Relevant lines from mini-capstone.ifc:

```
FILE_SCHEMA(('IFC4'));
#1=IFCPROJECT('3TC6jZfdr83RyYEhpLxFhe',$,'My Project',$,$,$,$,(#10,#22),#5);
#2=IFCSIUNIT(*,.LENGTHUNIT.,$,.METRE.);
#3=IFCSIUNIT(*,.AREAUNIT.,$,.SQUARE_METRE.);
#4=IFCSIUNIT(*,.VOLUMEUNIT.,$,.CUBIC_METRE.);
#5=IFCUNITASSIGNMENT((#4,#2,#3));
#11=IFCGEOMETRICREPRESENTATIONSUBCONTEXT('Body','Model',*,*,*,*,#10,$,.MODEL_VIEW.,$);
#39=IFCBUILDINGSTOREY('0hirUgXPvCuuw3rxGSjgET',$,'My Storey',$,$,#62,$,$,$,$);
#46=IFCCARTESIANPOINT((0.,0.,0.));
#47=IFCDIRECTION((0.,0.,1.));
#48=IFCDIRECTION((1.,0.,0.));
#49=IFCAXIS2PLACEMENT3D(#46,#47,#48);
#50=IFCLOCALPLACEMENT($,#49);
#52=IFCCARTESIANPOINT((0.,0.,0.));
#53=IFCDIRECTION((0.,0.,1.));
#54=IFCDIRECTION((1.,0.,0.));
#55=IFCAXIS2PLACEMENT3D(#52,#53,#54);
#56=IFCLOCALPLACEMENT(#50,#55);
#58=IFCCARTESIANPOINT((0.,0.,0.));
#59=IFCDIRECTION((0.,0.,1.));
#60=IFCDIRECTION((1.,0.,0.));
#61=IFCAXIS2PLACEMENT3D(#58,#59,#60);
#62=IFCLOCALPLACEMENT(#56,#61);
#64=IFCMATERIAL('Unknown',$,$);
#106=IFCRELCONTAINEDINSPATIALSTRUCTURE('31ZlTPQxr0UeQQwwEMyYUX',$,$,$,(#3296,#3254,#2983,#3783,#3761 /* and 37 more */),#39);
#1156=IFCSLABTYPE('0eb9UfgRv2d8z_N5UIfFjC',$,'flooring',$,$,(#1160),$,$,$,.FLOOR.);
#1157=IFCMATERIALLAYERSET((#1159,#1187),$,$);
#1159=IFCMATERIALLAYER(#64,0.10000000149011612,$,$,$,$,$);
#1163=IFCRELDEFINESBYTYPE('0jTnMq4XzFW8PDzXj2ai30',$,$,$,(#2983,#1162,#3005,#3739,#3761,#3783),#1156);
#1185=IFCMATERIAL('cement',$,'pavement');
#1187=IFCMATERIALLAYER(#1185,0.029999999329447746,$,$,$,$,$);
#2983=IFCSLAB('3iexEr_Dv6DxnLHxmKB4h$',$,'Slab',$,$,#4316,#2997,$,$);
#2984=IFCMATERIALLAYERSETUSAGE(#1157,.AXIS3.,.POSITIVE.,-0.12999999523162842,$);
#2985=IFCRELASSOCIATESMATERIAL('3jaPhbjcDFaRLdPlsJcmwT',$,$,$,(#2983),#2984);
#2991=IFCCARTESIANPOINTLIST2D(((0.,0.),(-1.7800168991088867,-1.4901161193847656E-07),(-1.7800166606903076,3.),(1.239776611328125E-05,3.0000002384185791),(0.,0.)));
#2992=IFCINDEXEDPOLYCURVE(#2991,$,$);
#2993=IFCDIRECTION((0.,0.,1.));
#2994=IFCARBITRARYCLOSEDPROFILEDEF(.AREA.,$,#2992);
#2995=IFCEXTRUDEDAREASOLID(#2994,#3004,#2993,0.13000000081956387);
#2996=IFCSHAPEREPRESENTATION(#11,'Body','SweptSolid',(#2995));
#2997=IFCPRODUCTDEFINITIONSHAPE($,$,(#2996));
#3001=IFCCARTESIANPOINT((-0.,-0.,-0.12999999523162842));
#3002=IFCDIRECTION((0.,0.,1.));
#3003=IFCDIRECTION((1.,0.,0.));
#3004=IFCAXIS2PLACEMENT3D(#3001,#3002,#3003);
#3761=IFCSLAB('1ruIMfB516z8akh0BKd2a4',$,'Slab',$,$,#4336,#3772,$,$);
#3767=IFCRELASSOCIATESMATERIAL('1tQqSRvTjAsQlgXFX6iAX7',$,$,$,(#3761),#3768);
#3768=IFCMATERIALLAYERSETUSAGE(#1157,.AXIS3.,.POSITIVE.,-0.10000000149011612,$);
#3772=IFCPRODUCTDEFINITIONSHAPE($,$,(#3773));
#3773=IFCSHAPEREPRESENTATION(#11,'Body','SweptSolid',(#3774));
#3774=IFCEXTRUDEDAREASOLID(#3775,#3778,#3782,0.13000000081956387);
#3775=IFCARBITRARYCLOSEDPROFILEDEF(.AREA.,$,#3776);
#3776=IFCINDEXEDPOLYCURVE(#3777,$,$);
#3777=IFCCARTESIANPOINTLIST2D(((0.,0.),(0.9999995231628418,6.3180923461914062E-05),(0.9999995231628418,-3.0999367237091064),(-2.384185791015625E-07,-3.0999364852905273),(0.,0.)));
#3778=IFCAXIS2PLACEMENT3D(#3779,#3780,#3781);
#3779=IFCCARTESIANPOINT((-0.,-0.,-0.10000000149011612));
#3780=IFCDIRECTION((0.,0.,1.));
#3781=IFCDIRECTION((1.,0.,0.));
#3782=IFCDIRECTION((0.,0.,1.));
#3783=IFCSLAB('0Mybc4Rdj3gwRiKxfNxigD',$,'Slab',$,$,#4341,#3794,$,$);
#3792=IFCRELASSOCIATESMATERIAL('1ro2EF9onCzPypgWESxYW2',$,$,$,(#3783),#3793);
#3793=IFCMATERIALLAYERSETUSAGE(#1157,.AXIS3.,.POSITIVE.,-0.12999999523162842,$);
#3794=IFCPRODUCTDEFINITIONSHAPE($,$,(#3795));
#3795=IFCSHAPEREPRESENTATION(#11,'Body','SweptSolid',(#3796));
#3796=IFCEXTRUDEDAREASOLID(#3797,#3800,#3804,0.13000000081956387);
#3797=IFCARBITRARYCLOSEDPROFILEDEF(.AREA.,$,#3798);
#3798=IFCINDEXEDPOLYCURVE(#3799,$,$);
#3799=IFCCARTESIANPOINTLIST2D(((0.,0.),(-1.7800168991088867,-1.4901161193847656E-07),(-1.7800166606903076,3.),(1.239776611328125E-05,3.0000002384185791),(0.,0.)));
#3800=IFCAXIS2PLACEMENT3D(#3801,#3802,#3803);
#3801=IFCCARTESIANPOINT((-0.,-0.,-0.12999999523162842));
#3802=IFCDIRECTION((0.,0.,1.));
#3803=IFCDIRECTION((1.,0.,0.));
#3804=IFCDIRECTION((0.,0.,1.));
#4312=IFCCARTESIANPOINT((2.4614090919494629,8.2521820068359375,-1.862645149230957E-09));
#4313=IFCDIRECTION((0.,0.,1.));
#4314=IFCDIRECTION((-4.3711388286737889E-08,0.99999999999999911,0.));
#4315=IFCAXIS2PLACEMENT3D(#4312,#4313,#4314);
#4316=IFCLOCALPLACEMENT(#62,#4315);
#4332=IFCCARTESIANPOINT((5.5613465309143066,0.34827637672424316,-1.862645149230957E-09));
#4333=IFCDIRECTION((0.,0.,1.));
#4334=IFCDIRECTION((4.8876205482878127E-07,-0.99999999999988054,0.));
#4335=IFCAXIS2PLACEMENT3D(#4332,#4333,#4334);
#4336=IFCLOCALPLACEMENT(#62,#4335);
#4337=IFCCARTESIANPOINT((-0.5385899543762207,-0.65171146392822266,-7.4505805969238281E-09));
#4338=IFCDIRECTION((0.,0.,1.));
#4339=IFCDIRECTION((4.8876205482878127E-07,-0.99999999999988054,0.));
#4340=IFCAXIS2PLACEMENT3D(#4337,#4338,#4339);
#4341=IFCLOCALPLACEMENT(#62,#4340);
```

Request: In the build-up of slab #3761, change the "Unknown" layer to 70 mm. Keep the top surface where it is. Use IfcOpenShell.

```python
import ifcopenshell
import ifcopenshell.util.element
import ifcopenshell.util.representation
import ifcopenshell.util.unit

model = ifcopenshell.open("mini-capstone.ifc")
unit_scale = ifcopenshell.util.unit.calculate_unit_scale(model)

layer_set = model.by_id(1157)
layer = next(l for l in layer_set.MaterialLayers if l.Material and l.Material.Name == "Unknown")
change = 0.07 / unit_scale - layer.LayerThickness
layer.LayerThickness += change

# The layer set is shared, so every slab that uses it gets the new thickness.
slabs = [e for e in ifcopenshell.util.element.get_elements_by_material(model, layer_set) if e.is_a("IfcSlab")]
for slab in sorted(slabs, key=lambda e: e.id()):
    body = ifcopenshell.util.representation.get_representation(slab, "Model", "Body")
    solid = body.Items[0]
    old_depth = solid.Depth
    solid.Depth += change
    # Extruded upwards: lower the start of the extrusion so the top stays.
    x, y, z = solid.Position.Location.Coordinates
    solid.Position.Location = model.createIfcCartesianPoint((x, y, z - change))
    print(slab.id(), f"{old_depth:g} -> {solid.Depth:g}")

# The layers are counted up from the underside, which has moved.
for usage in {ifcopenshell.util.element.get_material(slab) for slab in slabs}:
    usage.OffsetFromReferenceLine -= change

model.write("mini-capstone_rev.ifc")
```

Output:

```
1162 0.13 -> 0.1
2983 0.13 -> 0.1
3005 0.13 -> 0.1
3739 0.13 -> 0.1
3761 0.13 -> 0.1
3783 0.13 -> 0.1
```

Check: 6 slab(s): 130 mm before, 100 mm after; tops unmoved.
